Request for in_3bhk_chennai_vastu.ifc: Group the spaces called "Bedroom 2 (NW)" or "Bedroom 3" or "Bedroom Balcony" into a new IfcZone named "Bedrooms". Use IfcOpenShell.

First a look at what the model holds.

```python
import ifcopenshell

model = ifcopenshell.open("in_3bhk_chennai_vastu.ifc")
print(model.schema)
seen = {}
for space in model.by_type("IfcSpace"):
    seen[space.LongName] = seen.get(space.LongName, 0) + 1
for name, count in sorted(seen.items(), key=str):
    print(count, "x", name)
print("zones:", [z.Name for z in model.by_type("IfcZone")][:20])
```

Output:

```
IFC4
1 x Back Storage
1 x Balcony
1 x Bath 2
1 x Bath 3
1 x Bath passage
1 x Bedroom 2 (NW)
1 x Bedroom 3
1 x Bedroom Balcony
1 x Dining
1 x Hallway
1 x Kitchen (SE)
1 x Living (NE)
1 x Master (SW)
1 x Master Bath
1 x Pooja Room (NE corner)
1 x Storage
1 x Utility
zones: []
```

```python
import ifcopenshell
import ifcopenshell.api.group
import ifcopenshell.api.root

model = ifcopenshell.open("in_3bhk_chennai_vastu.ifc")

names = {"Bedroom 2 (NW)", "Bedroom 3", "Bedroom Balcony"}
spaces = [s for s in model.by_type("IfcSpace") if s.LongName in names]

zone = ifcopenshell.api.root.create_entity(model, ifc_class="IfcZone", name="Bedrooms")
ifcopenshell.api.group.assign_group(model, products=spaces, group=zone)
print(len(spaces), "spaces in", zone.Name)

model.write("in_3bhk_chennai_vastu_edited.ifc")
```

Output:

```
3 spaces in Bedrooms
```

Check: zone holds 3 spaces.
